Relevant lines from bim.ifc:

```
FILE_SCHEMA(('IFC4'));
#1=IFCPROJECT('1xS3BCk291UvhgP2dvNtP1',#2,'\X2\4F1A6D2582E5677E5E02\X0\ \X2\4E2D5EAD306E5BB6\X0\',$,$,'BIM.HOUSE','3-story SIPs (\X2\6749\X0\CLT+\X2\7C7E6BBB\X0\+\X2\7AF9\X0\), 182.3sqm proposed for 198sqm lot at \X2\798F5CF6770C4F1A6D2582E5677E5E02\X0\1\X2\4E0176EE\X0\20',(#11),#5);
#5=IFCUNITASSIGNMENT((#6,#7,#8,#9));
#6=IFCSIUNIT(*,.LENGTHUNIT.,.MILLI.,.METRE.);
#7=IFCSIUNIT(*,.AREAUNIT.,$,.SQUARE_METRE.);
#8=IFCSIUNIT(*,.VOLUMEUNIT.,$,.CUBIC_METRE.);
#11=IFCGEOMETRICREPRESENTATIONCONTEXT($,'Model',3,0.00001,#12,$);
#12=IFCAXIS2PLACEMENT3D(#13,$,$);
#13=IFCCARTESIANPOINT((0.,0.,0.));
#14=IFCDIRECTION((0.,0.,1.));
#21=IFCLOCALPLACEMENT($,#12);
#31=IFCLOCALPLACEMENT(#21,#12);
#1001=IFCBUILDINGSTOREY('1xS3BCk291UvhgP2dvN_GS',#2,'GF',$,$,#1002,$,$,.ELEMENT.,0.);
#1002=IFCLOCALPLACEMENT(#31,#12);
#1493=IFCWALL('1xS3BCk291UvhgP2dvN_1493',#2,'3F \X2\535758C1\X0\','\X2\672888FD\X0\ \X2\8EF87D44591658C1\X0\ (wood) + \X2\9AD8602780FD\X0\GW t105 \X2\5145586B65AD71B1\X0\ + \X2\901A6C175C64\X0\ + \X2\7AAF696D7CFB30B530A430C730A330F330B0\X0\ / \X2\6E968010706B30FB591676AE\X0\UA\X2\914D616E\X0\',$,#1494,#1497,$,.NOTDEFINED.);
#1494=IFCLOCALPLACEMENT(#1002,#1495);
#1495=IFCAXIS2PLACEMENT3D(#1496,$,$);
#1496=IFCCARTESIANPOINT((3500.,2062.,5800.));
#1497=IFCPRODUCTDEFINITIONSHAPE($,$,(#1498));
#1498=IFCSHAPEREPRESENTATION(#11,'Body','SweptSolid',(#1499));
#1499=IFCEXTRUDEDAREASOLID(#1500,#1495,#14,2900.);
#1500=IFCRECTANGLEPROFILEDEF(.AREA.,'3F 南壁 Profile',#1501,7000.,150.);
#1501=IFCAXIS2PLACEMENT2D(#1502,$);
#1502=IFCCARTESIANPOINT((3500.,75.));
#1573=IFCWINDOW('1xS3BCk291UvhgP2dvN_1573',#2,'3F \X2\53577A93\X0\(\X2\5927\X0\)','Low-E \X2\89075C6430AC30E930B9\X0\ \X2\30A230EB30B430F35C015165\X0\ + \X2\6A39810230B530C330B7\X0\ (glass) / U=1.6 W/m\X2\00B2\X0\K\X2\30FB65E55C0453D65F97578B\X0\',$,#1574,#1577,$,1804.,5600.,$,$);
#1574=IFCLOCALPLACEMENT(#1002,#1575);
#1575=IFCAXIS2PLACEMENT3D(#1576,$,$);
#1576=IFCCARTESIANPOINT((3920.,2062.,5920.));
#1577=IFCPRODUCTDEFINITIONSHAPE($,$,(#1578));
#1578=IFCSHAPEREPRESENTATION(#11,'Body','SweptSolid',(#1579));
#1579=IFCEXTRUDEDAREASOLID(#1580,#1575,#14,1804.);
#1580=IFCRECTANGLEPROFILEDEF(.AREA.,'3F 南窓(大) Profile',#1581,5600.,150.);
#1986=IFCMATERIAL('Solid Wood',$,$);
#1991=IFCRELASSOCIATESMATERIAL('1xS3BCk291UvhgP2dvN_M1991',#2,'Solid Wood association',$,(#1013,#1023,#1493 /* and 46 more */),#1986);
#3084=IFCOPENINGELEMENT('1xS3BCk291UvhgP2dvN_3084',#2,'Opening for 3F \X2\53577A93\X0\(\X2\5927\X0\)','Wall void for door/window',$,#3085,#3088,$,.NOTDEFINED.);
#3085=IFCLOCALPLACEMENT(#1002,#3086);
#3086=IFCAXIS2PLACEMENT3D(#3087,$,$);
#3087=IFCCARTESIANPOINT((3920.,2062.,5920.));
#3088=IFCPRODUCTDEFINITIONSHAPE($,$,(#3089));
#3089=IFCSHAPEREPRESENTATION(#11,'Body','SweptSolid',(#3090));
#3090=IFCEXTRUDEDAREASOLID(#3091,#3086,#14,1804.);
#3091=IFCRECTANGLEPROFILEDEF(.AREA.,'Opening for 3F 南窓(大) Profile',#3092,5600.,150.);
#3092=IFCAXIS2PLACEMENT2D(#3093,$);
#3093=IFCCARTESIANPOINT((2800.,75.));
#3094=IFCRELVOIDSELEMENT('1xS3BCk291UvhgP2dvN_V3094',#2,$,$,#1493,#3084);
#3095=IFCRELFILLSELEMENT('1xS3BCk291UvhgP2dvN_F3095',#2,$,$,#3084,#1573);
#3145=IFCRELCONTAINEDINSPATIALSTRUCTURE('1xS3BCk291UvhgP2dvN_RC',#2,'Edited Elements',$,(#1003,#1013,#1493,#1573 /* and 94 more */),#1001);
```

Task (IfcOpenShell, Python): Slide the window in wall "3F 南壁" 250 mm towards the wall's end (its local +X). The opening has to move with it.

```python
import ifcopenshell
import ifcopenshell.api.geometry
import ifcopenshell.util.placement

model = ifcopenshell.open("bim.ifc")

window = model.by_guid("1xS3BCk291UvhgP2dvN_1573")
opening = window.FillsVoids[0].RelatingOpeningElement
wall = opening.VoidsElements[0].RelatingBuildingElement

wall_matrix = ifcopenshell.util.placement.get_local_placement(wall.ObjectPlacement)
shift = wall_matrix[:3, 0] * 250.0
before = ifcopenshell.util.placement.get_local_placement(window.ObjectPlacement)[:3, 3].copy()

# The window is not placed relative to its opening, so move both.
for product in (opening, window):
    matrix = ifcopenshell.util.placement.get_local_placement(product.ObjectPlacement)
    matrix[:3, 3] += shift
    ifcopenshell.api.geometry.edit_object_placement(model, product=product, matrix=matrix, is_si=False)

after = ifcopenshell.util.placement.get_local_placement(window.ObjectPlacement)[:3, 3]
print("window moved by", (after - before).round(3) + 0.0)

model.write("bim-out.ifc")
```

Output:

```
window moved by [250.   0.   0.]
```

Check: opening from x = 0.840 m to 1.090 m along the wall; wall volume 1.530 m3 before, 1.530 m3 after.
